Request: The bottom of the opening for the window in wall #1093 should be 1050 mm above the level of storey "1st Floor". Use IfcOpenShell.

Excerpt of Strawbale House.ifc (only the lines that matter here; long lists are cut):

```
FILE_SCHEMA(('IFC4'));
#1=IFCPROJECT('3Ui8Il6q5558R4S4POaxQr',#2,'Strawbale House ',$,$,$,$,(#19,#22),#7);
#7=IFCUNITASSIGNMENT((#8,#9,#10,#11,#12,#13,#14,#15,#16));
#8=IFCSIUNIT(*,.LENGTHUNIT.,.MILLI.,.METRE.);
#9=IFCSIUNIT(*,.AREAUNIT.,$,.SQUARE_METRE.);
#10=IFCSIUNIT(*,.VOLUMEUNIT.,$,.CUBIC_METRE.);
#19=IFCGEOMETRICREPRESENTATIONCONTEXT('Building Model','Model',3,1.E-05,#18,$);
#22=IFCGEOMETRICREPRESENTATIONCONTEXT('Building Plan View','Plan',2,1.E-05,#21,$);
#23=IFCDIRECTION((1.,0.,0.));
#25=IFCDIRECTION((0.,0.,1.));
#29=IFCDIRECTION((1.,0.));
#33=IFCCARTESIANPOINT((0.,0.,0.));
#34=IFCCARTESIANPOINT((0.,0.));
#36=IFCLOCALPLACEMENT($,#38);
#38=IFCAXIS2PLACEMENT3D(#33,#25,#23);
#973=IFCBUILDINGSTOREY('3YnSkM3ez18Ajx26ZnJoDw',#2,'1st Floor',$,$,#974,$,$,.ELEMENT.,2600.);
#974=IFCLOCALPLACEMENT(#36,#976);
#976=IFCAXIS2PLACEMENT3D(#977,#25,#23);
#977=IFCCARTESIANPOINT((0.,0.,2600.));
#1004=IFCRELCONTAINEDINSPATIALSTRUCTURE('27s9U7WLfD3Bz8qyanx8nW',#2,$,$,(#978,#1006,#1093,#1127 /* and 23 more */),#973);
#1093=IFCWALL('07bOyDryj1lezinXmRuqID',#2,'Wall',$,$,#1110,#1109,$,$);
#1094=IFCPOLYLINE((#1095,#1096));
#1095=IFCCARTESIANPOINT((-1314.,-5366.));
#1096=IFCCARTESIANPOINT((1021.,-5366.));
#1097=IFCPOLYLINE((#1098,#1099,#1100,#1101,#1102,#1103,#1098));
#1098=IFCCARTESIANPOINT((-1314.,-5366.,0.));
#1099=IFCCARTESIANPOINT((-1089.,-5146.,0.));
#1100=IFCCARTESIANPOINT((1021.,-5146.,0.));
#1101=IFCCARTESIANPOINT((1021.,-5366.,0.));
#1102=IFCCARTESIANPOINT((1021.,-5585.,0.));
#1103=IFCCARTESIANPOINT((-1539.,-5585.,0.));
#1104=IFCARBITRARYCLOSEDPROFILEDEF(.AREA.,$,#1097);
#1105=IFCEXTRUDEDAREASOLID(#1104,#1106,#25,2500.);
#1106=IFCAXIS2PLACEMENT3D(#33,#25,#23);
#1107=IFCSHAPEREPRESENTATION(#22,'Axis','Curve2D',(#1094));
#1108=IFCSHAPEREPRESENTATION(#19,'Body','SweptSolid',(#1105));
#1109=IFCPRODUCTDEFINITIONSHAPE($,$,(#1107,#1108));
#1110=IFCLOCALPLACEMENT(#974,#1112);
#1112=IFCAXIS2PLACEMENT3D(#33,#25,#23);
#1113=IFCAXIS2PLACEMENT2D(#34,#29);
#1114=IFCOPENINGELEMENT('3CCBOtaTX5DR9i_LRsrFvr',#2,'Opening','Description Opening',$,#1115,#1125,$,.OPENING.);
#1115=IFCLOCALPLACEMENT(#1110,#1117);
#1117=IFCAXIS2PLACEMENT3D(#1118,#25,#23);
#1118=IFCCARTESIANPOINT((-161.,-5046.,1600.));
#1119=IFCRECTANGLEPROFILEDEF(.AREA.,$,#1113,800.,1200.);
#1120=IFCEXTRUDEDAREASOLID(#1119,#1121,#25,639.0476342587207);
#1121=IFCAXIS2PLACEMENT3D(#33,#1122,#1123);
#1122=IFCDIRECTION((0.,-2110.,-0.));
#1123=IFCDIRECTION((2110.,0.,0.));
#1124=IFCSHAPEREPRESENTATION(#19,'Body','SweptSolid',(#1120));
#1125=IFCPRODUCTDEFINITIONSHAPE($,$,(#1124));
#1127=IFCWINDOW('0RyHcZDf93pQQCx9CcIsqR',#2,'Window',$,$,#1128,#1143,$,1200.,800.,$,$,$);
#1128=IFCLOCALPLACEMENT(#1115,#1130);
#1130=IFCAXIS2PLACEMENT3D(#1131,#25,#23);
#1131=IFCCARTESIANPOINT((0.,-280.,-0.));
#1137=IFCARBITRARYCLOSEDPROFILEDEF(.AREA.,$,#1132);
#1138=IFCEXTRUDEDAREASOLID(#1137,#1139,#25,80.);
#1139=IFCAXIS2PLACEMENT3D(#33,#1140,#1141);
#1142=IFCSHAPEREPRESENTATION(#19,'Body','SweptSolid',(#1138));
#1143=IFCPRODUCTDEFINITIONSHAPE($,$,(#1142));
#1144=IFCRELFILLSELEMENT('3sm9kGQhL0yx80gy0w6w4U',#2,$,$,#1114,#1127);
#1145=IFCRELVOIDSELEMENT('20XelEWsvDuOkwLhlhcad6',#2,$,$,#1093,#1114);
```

```python
import numpy as np
import ifcopenshell
import ifcopenshell.api.geometry
import ifcopenshell.geom
import ifcopenshell.util.element
import ifcopenshell.util.placement
import ifcopenshell.util.shape
import ifcopenshell.util.unit

model = ifcopenshell.open("Strawbale House.ifc")
unit_scale = ifcopenshell.util.unit.calculate_unit_scale(model)

window = model.by_guid("0RyHcZDf93pQQCx9CcIsqR")
opening = window.FillsVoids[0].RelatingOpeningElement
storey = ifcopenshell.util.element.get_container(window, ifc_class="IfcBuildingStorey")
level = ifcopenshell.util.placement.get_local_placement(storey.ObjectPlacement)[2, 3]

# The opening's origin need not be at the sill, so measure its lowest point.
shape = ifcopenshell.geom.create_shape(ifcopenshell.geom.settings(), opening)
bottom = ifcopenshell.util.shape.get_shape_bottom_elevation(shape, shape.geometry) / unit_scale
dz = level + 1050.0 - bottom

shift = np.array([0.0, 0.0, dz])
# The window is placed relative to its opening, so it follows when the opening moves.
matrix = ifcopenshell.util.placement.get_local_placement(opening.ObjectPlacement)
matrix[:3, 3] += shift
ifcopenshell.api.geometry.edit_object_placement(
    model, product=opening, matrix=matrix, is_si=False, should_transform_children=True
)

print(f"moved by {dz * unit_scale:+.3f} m")

model.write("Strawbale House-out.ifc")
```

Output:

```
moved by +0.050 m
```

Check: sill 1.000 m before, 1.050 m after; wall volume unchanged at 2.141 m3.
